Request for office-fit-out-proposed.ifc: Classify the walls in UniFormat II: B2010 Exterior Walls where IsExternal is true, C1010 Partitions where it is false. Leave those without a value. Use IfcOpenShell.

First a look at what the model holds.

```python
import ifcopenshell
import ifcopenshell.util.element

model = ifcopenshell.open("office-fit-out-proposed.ifc")
print(model.schema)
print("classifications:", [c.Name for c in model.by_type("IfcClassification")])
values = [ifcopenshell.util.element.get_pset(e, "Pset_WallCommon", "IsExternal") for e in model.by_type("IfcWall")]
for value in (True, False, None):
    print("IsExternal", value, values.count(value))
```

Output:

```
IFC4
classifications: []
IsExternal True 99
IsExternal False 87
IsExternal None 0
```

```python
import ifcopenshell
import ifcopenshell.api.classification
import ifcopenshell.util.element

model = ifcopenshell.open("office-fit-out-proposed.ifc")

system = ifcopenshell.api.classification.add_classification(model, classification="UniFormat II")

walls = model.by_type("IfcWall")
external = {e: ifcopenshell.util.element.get_pset(e, "Pset_WallCommon", "IsExternal") for e in walls}
for flag, code, name in ((True, "B2010", "Exterior Walls"), (False, "C1010", "Partitions")):
    products = [e for e in walls if external[e] is flag]
    ifcopenshell.api.classification.add_reference(
        model, products=products, classification=system, identification=code, name=name
    )
    print(code, len(products))

model.write("office-fit-out-proposed_edited.ifc")
```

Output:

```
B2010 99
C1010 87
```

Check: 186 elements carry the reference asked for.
